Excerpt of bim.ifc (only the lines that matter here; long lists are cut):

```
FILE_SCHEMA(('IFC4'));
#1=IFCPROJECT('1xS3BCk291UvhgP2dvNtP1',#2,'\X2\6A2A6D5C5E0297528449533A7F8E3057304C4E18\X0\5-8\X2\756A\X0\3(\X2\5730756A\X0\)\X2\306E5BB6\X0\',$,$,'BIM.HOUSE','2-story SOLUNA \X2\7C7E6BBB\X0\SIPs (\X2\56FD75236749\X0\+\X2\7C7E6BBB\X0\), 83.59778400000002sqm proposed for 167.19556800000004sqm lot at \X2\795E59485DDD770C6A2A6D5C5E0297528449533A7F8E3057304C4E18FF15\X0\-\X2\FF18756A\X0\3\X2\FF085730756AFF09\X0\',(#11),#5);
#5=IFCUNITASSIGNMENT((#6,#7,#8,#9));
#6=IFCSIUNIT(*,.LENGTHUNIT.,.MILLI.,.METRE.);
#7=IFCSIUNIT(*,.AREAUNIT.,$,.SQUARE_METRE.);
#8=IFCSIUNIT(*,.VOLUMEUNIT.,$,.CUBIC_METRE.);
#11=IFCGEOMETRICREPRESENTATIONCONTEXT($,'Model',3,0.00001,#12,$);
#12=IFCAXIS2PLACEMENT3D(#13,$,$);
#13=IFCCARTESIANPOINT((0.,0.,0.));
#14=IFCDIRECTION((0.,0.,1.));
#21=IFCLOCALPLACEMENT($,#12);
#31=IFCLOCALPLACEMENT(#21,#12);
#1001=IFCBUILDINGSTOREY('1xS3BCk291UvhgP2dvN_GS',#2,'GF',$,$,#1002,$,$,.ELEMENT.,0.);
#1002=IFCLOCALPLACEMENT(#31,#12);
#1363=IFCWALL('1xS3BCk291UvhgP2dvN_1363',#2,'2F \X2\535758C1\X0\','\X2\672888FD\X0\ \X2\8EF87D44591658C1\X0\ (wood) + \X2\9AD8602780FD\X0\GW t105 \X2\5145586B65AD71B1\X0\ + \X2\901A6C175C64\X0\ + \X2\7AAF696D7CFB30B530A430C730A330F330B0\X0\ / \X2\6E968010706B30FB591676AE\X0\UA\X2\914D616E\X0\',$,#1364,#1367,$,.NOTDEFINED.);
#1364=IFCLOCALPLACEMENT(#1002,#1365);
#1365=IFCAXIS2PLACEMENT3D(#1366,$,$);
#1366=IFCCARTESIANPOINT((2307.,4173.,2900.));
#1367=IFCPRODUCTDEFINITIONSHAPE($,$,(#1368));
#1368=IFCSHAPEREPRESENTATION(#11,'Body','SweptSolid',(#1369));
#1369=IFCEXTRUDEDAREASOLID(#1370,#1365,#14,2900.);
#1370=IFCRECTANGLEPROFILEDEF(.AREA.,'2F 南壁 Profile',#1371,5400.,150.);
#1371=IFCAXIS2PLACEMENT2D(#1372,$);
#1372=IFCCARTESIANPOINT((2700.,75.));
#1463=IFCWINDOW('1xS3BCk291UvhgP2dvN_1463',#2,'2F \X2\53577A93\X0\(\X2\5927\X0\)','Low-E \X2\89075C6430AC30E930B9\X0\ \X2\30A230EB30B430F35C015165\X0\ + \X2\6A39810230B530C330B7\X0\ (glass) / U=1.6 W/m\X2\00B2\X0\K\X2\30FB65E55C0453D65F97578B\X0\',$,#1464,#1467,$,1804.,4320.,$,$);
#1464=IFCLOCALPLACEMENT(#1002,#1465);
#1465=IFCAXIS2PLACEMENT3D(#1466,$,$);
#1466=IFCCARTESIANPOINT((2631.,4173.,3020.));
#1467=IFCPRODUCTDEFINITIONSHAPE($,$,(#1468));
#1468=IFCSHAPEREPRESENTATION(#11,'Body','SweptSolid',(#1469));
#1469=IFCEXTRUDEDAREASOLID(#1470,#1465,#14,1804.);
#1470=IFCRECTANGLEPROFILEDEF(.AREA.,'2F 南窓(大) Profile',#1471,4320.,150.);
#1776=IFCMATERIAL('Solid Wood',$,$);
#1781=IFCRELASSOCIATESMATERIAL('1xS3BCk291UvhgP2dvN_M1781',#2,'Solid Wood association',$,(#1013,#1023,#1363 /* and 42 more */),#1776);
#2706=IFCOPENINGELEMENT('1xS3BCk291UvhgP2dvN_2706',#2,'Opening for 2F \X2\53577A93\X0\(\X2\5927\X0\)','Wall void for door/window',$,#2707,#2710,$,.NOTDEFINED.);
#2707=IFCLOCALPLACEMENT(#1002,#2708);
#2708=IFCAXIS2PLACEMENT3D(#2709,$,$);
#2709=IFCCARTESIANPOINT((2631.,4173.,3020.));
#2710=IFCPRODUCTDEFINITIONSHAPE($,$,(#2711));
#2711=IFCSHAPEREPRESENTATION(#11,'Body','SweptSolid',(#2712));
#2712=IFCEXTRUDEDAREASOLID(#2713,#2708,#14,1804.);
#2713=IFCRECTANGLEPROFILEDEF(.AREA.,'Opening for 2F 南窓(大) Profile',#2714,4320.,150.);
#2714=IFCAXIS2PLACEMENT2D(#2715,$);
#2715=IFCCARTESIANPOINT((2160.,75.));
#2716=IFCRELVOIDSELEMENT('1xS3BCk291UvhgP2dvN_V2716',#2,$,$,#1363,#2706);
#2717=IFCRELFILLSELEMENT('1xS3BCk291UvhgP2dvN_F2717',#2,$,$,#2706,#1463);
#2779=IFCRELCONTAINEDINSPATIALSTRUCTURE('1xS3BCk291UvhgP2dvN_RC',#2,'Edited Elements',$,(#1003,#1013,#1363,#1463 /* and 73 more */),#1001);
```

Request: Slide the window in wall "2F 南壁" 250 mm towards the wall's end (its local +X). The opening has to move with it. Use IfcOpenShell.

```python
import ifcopenshell
import ifcopenshell.api.geometry
import ifcopenshell.util.placement
import ifcopenshell.util.unit

model = ifcopenshell.open("bim.ifc")
unit_scale = ifcopenshell.util.unit.calculate_unit_scale(model)

window = model.by_id(1463)
opening = window.FillsVoids[0].RelatingOpeningElement
wall = opening.VoidsElements[0].RelatingBuildingElement

wall_matrix = ifcopenshell.util.placement.get_local_placement(wall.ObjectPlacement)
shift = wall_matrix[:3, 0] * 0.25 / unit_scale
before = ifcopenshell.util.placement.get_local_placement(window.ObjectPlacement)[:3, 3].copy()

# The window is not placed relative to its opening, so move both.
for product in (opening, window):
    matrix = ifcopenshell.util.placement.get_local_placement(product.ObjectPlacement)
    matrix[:3, 3] += shift
    ifcopenshell.api.geometry.edit_object_placement(model, product=product, matrix=matrix, is_si=False)

after = ifcopenshell.util.placement.get_local_placement(window.ObjectPlacement)[:3, 3]
print("window moved by", (after - before).round(3) + 0.0)

model.write("bim_edited.ifc")
```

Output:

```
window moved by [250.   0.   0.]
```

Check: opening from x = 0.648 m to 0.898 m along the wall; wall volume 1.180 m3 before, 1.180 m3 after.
